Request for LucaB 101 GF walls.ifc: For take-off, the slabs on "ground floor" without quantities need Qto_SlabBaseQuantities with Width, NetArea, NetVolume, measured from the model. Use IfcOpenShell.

First a look at what the model holds.

```python
import ifcopenshell
import ifcopenshell.util.element
import ifcopenshell.util.unit

model = ifcopenshell.open("LucaB 101 GF walls.ifc")
print(model.schema)
for unit_type in ("LENGTHUNIT", "AREAUNIT", "VOLUMEUNIT"):
    print(unit_type, ifcopenshell.util.unit.calculate_unit_scale(model, unit_type))
storey = next(s for s in model.by_type("IfcBuildingStorey") if s.Name == "ground floor")
slabs = [e for e in ifcopenshell.util.element.get_decomposition(storey) if e.is_a("IfcSlab")]
for e in sorted(slabs, key=lambda e: e.id()):
    print(e.id(), e.is_a(), e.Name, list(ifcopenshell.util.element.get_psets(e, qtos_only=True)), sep=" | ")
```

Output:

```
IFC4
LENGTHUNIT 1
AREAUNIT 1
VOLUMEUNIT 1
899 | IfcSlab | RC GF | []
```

```python
import ifcopenshell
import ifcopenshell.api.pset
import ifcopenshell.geom
import ifcopenshell.util.element
import ifcopenshell.util.shape
import ifcopenshell.util.unit

model = ifcopenshell.open("LucaB 101 GF walls.ifc")
unit_scale = ifcopenshell.util.unit.calculate_unit_scale(model)
area_scale = ifcopenshell.util.unit.calculate_unit_scale(model, "AREAUNIT")
volume_scale = ifcopenshell.util.unit.calculate_unit_scale(model, "VOLUMEUNIT")
settings = ifcopenshell.geom.settings()

storey = next(s for s in model.by_type("IfcBuildingStorey") if s.Name == "ground floor")
slabs = [e for e in ifcopenshell.util.element.get_decomposition(storey) if e.is_a("IfcSlab")]

for e in sorted(slabs, key=lambda e: e.id()):
    if ifcopenshell.util.element.get_psets(e, qtos_only=True, should_inherit=False):
        continue
    # Geometry comes back in metres, in the element's own axes.
    shape = ifcopenshell.geom.create_shape(settings, e)
    values = {
        "Width": ifcopenshell.util.shape.get_z(shape.geometry) / unit_scale,
        "NetArea": ifcopenshell.util.shape.get_footprint_area(shape.geometry) / area_scale,
        "NetVolume": ifcopenshell.util.shape.get_volume(shape.geometry) / volume_scale,
    }
    qto = ifcopenshell.api.pset.add_qto(model, product=e, name="Qto_SlabBaseQuantities")
    ifcopenshell.api.pset.edit_qto(model, qto=qto, properties=values)
    print(e.id(), {k: round(v, 3) for k, v in values.items()})

model.write("LucaB 101 GF walls_edited.ifc")
```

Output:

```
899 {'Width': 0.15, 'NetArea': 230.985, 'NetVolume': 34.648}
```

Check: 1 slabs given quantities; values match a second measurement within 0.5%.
